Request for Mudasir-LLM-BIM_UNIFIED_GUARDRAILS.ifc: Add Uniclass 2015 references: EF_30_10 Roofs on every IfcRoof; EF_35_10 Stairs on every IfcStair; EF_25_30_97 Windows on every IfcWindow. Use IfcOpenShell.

First a look at what the model holds.

```python
import ifcopenshell

model = ifcopenshell.open("Mudasir-LLM-BIM_UNIFIED_GUARDRAILS.ifc")
print(model.schema)
print("classifications:", [c.Name for c in model.by_type("IfcClassification")])
for ifc_class in ("IfcDoor", "IfcRoof", "IfcStair", "IfcWall", "IfcWindow"):
    print(ifc_class, len(model.by_type(ifc_class)))
```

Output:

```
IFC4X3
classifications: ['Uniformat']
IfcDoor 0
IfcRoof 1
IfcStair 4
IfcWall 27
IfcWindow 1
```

```python
import ifcopenshell
import ifcopenshell.api.classification

model = ifcopenshell.open("Mudasir-LLM-BIM_UNIFIED_GUARDRAILS.ifc")

system = ifcopenshell.api.classification.add_classification(model, classification="Uniclass 2015")

codes = {
    "IfcRoof": ("EF_30_10", "Roofs"),
    "IfcStair": ("EF_35_10", "Stairs"),
    "IfcWindow": ("EF_25_30_97", "Windows"),
}
for ifc_class, (code, name) in codes.items():
    products = model.by_type(ifc_class)
    ifcopenshell.api.classification.add_reference(
        model, products=products, classification=system, identification=code, name=name
    )
    print(code, len(products))

model.write("Mudasir-LLM-BIM_UNIFIED_GUARDRAILS-out.ifc")
```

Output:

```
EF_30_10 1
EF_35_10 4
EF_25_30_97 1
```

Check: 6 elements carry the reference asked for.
